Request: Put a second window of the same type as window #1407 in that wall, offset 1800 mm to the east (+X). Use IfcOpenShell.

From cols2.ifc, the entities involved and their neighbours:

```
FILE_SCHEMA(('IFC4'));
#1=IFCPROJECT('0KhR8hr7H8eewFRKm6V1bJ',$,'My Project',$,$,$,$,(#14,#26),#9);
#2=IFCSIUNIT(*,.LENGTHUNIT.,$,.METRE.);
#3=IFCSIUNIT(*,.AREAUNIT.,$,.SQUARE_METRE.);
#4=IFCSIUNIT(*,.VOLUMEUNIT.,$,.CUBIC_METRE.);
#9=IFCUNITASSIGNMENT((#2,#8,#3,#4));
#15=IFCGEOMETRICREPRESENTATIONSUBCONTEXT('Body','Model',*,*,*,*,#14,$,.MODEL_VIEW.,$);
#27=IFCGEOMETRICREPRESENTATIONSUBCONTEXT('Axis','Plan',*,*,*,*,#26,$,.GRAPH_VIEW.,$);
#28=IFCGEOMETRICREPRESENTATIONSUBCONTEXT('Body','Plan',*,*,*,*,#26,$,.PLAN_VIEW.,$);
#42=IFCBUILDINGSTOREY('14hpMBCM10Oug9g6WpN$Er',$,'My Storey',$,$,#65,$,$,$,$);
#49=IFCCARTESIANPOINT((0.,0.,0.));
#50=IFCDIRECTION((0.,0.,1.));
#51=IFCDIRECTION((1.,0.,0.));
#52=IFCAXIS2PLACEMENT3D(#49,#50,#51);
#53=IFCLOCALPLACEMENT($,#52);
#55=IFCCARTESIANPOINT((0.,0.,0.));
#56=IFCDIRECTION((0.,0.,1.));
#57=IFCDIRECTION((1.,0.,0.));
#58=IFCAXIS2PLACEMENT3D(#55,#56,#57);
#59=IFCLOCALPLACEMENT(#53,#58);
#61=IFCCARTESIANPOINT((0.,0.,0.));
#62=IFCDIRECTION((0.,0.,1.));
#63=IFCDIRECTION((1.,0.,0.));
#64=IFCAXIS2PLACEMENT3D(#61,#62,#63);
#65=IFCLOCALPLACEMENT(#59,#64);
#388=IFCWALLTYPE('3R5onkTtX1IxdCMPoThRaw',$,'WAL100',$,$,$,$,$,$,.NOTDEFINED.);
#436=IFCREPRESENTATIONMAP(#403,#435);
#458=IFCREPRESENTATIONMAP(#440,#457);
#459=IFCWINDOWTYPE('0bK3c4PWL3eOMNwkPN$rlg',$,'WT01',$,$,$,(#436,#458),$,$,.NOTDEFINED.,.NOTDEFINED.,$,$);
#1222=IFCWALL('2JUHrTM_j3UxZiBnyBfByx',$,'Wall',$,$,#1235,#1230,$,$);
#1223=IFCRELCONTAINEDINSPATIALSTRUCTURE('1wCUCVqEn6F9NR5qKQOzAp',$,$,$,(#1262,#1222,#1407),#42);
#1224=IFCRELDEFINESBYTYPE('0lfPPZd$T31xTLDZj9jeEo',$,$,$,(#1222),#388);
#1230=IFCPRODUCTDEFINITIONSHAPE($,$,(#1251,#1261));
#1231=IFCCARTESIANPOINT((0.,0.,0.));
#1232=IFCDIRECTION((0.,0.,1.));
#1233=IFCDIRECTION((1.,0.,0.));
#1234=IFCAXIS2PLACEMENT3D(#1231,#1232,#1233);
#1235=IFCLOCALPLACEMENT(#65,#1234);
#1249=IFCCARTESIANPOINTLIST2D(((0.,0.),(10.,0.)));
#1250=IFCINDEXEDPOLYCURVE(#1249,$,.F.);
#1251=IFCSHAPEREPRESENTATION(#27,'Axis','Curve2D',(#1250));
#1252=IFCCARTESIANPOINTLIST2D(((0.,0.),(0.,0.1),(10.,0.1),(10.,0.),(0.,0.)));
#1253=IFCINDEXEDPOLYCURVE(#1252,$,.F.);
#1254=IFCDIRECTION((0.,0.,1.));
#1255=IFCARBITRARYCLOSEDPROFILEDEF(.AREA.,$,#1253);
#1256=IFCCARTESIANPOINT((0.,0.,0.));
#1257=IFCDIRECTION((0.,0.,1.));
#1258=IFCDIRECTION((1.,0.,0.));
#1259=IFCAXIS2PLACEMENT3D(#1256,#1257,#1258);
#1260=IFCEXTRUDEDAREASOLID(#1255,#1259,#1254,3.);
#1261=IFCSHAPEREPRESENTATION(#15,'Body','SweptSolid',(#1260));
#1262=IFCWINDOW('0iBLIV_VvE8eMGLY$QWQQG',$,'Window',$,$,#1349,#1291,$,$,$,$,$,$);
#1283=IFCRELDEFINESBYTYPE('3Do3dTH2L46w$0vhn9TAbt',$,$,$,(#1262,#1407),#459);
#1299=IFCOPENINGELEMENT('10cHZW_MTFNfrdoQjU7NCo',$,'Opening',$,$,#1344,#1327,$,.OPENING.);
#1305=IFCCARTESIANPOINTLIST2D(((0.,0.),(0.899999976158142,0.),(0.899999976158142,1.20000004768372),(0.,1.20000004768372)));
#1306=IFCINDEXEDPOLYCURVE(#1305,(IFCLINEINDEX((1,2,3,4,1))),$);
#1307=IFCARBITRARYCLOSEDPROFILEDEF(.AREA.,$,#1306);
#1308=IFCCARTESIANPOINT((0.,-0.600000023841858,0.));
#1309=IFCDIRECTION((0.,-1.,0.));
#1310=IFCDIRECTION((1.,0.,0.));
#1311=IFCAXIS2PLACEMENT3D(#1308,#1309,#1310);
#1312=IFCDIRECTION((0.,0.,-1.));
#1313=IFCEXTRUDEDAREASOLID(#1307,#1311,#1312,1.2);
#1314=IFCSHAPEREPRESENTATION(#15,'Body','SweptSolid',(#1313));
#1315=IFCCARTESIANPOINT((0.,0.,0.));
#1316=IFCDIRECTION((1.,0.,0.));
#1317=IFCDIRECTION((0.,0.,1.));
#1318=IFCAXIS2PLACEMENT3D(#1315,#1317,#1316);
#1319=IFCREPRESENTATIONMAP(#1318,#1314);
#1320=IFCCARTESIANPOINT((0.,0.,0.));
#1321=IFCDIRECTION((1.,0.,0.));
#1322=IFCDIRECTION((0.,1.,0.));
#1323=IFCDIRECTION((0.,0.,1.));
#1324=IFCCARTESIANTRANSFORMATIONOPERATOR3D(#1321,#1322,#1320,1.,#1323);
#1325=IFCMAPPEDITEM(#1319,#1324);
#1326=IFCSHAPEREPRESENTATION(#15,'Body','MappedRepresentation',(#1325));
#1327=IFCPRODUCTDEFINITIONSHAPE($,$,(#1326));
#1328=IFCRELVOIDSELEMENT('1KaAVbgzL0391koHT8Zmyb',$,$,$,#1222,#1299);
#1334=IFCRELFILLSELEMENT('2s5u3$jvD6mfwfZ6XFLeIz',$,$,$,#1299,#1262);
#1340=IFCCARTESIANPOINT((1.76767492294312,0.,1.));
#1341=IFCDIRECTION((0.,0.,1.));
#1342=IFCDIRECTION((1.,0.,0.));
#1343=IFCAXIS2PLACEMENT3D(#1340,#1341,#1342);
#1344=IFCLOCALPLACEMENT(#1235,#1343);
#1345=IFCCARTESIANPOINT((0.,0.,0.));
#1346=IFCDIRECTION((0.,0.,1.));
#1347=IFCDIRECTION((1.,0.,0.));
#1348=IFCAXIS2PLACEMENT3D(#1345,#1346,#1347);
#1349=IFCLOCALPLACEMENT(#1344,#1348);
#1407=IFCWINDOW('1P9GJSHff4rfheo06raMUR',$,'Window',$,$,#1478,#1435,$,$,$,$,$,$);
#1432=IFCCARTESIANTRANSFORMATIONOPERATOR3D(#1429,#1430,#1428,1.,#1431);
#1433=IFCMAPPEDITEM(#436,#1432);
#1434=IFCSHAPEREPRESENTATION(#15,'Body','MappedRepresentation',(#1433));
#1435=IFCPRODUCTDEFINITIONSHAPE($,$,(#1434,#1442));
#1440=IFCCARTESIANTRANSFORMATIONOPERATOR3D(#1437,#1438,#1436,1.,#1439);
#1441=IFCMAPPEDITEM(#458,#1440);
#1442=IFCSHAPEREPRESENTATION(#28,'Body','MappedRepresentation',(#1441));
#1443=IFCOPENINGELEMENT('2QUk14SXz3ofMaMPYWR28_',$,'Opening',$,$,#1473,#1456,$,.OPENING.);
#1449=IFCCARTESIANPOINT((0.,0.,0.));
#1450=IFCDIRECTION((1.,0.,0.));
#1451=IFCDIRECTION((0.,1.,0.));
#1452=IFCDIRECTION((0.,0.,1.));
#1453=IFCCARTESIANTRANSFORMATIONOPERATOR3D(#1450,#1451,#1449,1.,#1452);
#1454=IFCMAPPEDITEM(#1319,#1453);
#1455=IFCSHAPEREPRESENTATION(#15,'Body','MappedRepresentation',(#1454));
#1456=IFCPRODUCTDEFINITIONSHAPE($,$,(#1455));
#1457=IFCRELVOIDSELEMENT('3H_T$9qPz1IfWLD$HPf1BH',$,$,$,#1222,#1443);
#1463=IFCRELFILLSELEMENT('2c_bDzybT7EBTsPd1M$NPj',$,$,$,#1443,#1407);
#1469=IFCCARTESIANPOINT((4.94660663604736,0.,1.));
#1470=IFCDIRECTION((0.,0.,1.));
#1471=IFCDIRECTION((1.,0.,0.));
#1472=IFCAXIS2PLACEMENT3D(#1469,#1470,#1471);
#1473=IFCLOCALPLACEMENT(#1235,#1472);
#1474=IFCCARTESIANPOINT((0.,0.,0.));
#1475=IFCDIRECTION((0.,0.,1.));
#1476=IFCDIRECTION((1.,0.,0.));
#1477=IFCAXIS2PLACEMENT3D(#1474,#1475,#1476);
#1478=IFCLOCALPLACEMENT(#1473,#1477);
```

```python
import ifcopenshell
import ifcopenshell.api.feature
import ifcopenshell.api.geometry
import ifcopenshell.api.root
import ifcopenshell.geom
import ifcopenshell.util.element
import ifcopenshell.util.placement
import ifcopenshell.util.shape
import ifcopenshell.util.unit

model = ifcopenshell.open("cols2.ifc")
unit_scale = ifcopenshell.util.unit.calculate_unit_scale(model)
settings = ifcopenshell.geom.settings()


def volume(element):
    """Net volume in cubic metres, openings subtracted."""
    shape = ifcopenshell.geom.create_shape(settings, element)
    return ifcopenshell.util.shape.get_volume(shape.geometry)


window = model.by_guid("1P9GJSHff4rfheo06raMUR")
opening = window.FillsVoids[0].RelatingOpeningElement
wall = opening.VoidsElements[0].RelatingBuildingElement
before = volume(wall)
shift = ifcopenshell.util.placement.get_local_placement(wall.ObjectPlacement)[:3, 0] * 1.8 / unit_scale

# copy_class copies the void relationship, type, container and properties, but no geometry.
new_opening = ifcopenshell.api.root.copy_class(model, product=opening)
new_opening.Representation = ifcopenshell.util.element.copy_deep(
    model, opening.Representation, exclude=["IfcGeometricRepresentationContext", "IfcRepresentationMap"]
)
new_window = ifcopenshell.api.root.copy_class(model, product=window)
new_window.Representation = ifcopenshell.util.element.copy_deep(
    model, window.Representation, exclude=["IfcGeometricRepresentationContext", "IfcRepresentationMap"]
)
ifcopenshell.api.feature.add_filling(model, opening=new_opening, element=new_window)

for old, new in ((opening, new_opening), (window, new_window)):
    matrix = ifcopenshell.util.placement.get_local_placement(old.ObjectPlacement)
    matrix[:3, 3] += shift
    ifcopenshell.api.geometry.edit_object_placement(model, product=new, matrix=matrix, is_si=False)

after = volume(wall)

print(f"wall volume {before:.3f} -> {after:.3f} m3")

model.write("cols2_updated.ifc")
```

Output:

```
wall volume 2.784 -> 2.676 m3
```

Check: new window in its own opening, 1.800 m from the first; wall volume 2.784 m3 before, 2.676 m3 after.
